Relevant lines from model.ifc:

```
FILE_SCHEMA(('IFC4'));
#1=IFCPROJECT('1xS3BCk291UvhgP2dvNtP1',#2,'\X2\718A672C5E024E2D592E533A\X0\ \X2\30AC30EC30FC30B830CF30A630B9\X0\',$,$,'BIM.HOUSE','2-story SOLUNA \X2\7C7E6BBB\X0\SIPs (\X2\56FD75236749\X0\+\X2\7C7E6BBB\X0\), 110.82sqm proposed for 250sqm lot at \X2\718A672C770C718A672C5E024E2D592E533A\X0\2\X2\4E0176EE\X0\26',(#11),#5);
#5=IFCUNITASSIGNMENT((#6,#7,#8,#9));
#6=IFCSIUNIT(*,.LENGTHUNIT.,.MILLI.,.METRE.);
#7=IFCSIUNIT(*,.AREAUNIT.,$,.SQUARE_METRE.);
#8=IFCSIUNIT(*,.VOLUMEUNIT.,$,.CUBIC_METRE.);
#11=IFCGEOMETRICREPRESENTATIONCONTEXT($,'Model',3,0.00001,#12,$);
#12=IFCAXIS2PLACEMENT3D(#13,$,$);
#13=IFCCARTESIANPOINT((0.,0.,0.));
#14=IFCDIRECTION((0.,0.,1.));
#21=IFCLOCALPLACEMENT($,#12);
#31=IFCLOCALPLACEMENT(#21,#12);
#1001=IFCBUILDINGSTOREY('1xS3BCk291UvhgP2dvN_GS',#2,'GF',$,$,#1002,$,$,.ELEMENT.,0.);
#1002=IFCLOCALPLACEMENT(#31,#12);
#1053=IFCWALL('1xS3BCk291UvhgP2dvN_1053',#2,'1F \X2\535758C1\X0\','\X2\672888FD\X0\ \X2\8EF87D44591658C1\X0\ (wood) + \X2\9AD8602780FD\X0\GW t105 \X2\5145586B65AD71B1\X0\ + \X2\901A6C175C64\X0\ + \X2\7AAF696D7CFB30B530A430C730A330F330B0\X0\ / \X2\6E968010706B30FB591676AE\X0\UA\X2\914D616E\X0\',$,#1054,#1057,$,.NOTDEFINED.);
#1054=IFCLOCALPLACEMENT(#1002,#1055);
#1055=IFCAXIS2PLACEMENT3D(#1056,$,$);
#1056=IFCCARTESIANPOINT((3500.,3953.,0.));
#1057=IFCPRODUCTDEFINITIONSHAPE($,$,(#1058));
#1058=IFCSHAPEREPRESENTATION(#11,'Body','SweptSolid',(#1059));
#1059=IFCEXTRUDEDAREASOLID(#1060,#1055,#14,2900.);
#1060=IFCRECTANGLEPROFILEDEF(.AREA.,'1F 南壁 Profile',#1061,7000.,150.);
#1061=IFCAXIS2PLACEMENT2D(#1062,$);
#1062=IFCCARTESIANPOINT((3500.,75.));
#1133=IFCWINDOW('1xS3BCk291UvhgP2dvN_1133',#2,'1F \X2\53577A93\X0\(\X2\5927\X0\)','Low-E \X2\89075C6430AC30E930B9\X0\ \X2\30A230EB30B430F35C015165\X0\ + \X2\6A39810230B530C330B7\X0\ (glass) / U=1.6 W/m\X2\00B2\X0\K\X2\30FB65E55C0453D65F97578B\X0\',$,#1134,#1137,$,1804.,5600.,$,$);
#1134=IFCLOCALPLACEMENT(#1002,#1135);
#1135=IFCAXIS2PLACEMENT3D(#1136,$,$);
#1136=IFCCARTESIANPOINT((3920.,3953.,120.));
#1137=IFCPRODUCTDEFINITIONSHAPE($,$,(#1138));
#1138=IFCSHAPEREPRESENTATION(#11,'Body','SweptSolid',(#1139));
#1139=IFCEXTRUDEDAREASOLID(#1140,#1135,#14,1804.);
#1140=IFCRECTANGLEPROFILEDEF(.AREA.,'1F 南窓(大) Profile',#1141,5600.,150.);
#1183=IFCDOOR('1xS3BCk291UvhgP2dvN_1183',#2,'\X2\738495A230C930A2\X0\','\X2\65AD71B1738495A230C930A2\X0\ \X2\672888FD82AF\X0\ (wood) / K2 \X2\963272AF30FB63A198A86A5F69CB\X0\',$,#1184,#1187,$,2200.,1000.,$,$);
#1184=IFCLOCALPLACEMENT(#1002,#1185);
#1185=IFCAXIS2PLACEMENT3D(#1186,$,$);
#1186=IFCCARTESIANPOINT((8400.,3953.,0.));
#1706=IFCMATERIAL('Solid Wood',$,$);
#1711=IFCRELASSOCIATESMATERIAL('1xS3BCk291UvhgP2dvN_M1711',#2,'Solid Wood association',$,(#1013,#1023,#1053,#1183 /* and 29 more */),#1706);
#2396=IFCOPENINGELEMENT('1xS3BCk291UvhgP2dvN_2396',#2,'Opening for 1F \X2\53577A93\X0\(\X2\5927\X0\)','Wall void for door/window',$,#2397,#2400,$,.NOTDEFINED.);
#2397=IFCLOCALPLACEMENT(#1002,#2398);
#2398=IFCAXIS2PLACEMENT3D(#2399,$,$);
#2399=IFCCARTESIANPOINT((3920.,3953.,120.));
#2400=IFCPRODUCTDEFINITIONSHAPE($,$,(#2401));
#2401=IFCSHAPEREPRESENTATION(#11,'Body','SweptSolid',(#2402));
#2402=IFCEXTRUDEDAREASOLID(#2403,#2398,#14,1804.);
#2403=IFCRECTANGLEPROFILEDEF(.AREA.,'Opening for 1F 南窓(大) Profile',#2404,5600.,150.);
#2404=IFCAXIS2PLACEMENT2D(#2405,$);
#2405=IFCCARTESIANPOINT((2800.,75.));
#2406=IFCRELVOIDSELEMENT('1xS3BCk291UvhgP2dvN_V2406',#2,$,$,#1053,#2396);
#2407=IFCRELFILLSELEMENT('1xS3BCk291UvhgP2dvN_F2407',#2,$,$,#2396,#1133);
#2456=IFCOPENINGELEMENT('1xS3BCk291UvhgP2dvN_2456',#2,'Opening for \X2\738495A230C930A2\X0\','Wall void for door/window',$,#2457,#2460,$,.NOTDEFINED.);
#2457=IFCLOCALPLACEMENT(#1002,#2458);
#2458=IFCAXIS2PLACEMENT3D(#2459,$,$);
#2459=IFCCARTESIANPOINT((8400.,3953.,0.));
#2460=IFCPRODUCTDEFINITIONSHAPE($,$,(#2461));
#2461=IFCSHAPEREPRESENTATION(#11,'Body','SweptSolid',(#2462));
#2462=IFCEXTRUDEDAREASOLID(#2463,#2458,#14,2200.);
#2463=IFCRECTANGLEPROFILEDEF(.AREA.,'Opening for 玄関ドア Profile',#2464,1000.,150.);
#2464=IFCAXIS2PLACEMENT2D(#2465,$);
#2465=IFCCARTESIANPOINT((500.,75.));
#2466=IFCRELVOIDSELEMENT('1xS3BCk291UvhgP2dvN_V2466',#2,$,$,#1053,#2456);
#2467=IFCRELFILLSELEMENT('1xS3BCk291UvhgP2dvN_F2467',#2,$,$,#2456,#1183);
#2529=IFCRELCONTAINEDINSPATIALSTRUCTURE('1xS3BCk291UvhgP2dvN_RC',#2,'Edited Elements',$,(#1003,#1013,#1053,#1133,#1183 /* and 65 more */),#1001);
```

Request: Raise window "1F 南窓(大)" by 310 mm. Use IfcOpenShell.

```python
import numpy as np
import ifcopenshell
import ifcopenshell.api.geometry
import ifcopenshell.util.placement
import ifcopenshell.util.unit

model = ifcopenshell.open("model.ifc")
unit_scale = ifcopenshell.util.unit.calculate_unit_scale(model)

window = model.by_id(1133)
opening = window.FillsVoids[0].RelatingOpeningElement
dz = 0.31 / unit_scale

shift = np.array([0.0, 0.0, dz])
# The window is not placed relative to its opening, so move both.
for product in (opening, window):
    matrix = ifcopenshell.util.placement.get_local_placement(product.ObjectPlacement)
    matrix[:3, 3] += shift
    ifcopenshell.api.geometry.edit_object_placement(model, product=product, matrix=matrix, is_si=False)

print(f"moved by {dz * unit_scale:+.3f} m")

model.write("model_edited.ifc")
```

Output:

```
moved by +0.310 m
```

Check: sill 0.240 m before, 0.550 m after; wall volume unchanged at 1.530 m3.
